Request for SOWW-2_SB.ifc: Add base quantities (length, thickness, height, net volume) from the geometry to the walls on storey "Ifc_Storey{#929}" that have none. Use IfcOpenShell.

First a look at what the model holds.

```python
import ifcopenshell
import ifcopenshell.util.element
import ifcopenshell.util.unit

model = ifcopenshell.open("SOWW-2_SB.ifc")
print(model.schema)
for unit_type in ("LENGTHUNIT", "AREAUNIT", "VOLUMEUNIT"):
    print(unit_type, ifcopenshell.util.unit.calculate_unit_scale(model, unit_type))
storey = next(s for s in model.by_type("IfcBuildingStorey") if s.Name == "Ifc_Storey{#929}")
walls = [e for e in ifcopenshell.util.element.get_decomposition(storey) if e.is_a("IfcWall")]
for e in sorted(walls, key=lambda e: e.id()):
    print(e.id(), e.is_a(), e.Name, list(ifcopenshell.util.element.get_psets(e, qtos_only=True)), sep=" | ")
```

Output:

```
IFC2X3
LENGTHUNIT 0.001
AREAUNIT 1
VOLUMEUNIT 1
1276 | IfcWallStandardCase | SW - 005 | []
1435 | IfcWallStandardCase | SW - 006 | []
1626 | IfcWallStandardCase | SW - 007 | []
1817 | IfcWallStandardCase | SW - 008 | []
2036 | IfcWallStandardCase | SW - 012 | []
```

```python
import ifcopenshell
import ifcopenshell.api.pset
import ifcopenshell.geom
import ifcopenshell.util.element
import ifcopenshell.util.shape
import ifcopenshell.util.unit

model = ifcopenshell.open("SOWW-2_SB.ifc")
unit_scale = ifcopenshell.util.unit.calculate_unit_scale(model)
volume_scale = ifcopenshell.util.unit.calculate_unit_scale(model, "VOLUMEUNIT")
settings = ifcopenshell.geom.settings()

storey = next(s for s in model.by_type("IfcBuildingStorey") if s.Name == "Ifc_Storey{#929}")
walls = [e for e in ifcopenshell.util.element.get_decomposition(storey) if e.is_a("IfcWall")]

for e in sorted(walls, key=lambda e: e.id()):
    if ifcopenshell.util.element.get_psets(e, qtos_only=True, should_inherit=False):
        continue
    # Geometry comes back in metres, in the element's own axes.
    shape = ifcopenshell.geom.create_shape(settings, e)
    values = {
        "Length": ifcopenshell.util.shape.get_x(shape.geometry) / unit_scale,
        "Width": ifcopenshell.util.shape.get_y(shape.geometry) / unit_scale,
        "Height": ifcopenshell.util.shape.get_z(shape.geometry) / unit_scale,
        "NetVolume": ifcopenshell.util.shape.get_volume(shape.geometry) / volume_scale,
    }
    qto = ifcopenshell.api.pset.add_qto(model, product=e, name="BaseQuantities")
    ifcopenshell.api.pset.edit_qto(model, qto=qto, properties=values)
    print(e.id(), {k: round(v, 3) for k, v in values.items()})

model.write("SOWW-2_SB-out.ifc")
```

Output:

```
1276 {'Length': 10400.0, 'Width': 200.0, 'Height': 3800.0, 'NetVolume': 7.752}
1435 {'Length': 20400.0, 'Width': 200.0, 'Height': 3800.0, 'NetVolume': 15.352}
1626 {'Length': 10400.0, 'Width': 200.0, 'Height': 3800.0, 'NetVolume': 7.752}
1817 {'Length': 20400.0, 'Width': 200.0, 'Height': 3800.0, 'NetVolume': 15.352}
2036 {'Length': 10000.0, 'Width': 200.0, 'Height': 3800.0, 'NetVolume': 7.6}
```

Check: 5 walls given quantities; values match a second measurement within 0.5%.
